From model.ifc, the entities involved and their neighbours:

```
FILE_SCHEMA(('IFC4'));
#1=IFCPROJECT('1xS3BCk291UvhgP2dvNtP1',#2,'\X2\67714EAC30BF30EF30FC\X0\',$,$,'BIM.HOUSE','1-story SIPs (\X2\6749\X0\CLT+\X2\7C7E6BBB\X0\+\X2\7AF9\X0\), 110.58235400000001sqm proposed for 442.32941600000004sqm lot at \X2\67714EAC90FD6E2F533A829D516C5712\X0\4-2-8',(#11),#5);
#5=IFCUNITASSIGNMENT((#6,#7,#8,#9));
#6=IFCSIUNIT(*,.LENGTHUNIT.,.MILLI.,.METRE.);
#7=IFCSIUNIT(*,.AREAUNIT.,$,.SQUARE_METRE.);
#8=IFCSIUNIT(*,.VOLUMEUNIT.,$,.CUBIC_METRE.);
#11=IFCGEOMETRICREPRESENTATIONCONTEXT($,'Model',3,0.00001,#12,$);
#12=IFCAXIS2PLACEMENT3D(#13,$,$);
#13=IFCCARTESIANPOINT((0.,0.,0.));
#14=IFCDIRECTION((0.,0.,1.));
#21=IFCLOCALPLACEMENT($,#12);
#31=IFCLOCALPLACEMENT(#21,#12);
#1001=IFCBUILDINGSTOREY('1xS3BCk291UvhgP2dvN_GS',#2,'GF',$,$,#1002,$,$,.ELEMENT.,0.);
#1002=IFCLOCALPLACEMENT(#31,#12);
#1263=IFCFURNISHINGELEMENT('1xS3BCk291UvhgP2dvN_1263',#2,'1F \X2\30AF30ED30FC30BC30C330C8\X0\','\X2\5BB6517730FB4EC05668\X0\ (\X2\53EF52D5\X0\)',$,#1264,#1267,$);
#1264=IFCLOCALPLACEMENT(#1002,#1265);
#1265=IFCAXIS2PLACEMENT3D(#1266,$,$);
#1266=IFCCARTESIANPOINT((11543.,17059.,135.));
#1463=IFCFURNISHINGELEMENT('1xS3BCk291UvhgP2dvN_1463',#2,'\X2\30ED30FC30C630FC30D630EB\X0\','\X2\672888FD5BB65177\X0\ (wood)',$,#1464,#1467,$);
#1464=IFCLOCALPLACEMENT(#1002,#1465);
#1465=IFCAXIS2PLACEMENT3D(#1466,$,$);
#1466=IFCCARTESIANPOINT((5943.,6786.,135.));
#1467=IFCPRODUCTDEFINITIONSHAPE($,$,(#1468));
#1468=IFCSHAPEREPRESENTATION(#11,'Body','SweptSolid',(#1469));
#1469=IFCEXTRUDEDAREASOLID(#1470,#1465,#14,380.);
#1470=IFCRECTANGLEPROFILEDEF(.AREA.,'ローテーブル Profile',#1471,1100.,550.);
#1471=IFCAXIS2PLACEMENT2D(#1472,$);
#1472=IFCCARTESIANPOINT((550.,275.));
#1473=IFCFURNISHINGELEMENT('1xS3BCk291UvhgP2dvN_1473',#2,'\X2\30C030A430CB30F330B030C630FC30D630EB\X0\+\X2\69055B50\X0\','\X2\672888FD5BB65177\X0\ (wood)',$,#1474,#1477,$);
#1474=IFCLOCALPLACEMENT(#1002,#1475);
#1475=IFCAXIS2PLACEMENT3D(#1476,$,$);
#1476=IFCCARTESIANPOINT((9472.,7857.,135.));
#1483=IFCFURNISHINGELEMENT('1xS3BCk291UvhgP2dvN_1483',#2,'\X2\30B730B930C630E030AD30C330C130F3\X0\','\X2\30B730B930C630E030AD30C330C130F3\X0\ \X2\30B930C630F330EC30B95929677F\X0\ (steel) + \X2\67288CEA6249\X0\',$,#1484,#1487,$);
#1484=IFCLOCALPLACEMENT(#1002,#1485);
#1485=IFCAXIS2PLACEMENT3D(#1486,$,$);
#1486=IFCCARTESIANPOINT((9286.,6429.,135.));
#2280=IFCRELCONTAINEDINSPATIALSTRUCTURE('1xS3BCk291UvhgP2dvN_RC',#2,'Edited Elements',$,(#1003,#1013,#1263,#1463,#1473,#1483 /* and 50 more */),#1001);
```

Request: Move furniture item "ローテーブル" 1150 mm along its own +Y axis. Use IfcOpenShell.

```python
import ifcopenshell
import ifcopenshell.api.geometry
import ifcopenshell.util.placement
import ifcopenshell.util.unit

model = ifcopenshell.open("model.ifc")
unit_scale = ifcopenshell.util.unit.calculate_unit_scale(model)

item = model.by_guid("1xS3BCk291UvhgP2dvN_1463")
matrix = ifcopenshell.util.placement.get_local_placement(item.ObjectPlacement)
matrix[:3, 3] += matrix[:3, 1] * 1.15 / unit_scale
ifcopenshell.api.geometry.edit_object_placement(model, product=item, matrix=matrix, is_si=False)

print(ifcopenshell.util.placement.get_local_placement(item.ObjectPlacement).round(3) + 0.0)

model.write("model_edited.ifc")
```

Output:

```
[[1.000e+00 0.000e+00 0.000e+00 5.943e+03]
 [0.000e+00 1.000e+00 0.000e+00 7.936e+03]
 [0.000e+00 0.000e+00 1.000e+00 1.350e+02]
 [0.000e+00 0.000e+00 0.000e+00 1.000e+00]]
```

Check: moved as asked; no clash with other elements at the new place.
